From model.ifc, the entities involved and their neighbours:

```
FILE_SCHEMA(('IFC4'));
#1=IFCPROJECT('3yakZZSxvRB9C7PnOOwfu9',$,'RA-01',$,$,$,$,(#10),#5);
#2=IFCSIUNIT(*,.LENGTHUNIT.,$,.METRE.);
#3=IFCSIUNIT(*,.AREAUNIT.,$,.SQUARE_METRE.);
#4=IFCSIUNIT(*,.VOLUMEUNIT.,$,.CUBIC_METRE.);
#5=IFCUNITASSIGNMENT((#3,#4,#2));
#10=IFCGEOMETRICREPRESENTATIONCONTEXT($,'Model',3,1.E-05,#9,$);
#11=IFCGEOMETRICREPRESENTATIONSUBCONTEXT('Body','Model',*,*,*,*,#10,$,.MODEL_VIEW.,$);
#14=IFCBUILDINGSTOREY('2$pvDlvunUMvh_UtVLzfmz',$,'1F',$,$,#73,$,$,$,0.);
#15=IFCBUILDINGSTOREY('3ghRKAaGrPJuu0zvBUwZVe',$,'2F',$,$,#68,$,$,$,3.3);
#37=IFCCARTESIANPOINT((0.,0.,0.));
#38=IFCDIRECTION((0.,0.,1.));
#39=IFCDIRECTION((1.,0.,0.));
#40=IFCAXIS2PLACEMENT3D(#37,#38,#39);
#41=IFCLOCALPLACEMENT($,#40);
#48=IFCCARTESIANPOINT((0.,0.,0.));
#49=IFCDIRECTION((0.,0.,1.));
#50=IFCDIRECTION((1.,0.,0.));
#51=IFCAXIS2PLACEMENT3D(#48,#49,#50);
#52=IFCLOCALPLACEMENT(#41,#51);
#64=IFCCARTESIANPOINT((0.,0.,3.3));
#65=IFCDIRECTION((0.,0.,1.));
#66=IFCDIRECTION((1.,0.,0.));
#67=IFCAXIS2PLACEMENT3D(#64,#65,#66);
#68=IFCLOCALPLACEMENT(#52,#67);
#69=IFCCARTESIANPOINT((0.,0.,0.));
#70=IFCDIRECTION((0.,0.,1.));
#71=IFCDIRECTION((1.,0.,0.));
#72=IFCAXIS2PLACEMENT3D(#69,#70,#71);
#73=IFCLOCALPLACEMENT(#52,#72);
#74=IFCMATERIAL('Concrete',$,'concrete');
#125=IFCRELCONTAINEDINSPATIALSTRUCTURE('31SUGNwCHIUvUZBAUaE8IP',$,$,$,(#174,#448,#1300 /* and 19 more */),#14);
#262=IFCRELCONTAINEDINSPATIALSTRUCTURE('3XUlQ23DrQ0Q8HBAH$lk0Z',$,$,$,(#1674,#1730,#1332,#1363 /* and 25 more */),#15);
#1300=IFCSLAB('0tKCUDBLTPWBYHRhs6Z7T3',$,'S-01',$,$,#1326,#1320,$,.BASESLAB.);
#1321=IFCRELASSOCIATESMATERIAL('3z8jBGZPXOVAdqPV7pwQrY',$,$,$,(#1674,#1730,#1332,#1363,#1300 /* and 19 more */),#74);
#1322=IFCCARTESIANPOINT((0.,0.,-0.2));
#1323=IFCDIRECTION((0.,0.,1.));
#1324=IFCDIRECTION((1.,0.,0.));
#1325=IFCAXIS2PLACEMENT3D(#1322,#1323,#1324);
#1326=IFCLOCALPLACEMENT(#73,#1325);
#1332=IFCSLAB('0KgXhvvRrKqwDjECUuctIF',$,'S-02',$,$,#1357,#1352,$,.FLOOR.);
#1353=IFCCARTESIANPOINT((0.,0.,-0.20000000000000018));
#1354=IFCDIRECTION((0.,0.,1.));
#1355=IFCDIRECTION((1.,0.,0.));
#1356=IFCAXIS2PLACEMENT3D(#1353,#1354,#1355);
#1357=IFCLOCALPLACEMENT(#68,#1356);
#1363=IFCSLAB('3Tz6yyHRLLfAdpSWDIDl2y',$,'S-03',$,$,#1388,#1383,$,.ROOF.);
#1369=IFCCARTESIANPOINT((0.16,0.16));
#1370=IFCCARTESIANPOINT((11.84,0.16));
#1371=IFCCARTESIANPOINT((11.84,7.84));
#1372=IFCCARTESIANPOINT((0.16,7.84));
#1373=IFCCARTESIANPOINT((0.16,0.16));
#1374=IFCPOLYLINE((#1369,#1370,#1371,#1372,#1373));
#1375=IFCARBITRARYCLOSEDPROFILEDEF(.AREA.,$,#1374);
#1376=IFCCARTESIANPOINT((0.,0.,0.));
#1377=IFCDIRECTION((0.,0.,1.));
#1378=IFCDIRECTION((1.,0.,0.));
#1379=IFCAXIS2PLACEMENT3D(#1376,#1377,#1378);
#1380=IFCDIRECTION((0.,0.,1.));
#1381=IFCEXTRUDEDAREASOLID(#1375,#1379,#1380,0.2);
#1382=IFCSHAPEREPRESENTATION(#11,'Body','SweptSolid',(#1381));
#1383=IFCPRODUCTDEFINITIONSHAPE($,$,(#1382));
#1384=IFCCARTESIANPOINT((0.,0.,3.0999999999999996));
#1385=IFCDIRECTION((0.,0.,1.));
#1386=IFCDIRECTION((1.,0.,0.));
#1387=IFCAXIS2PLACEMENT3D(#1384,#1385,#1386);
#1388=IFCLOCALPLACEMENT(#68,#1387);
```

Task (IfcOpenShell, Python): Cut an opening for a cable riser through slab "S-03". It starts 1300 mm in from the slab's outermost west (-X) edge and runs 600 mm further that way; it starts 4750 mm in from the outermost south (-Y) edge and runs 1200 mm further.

```python
import numpy as np
import ifcopenshell
import ifcopenshell.api.feature
import ifcopenshell.api.geometry
import ifcopenshell.api.root
import ifcopenshell.geom
import ifcopenshell.util.placement
import ifcopenshell.util.representation
import ifcopenshell.util.shape
import ifcopenshell.util.unit

model = ifcopenshell.open("model.ifc")
unit_scale = ifcopenshell.util.unit.calculate_unit_scale(model)
settings = ifcopenshell.geom.settings()


def volume(element):
    """Net volume in cubic metres, openings subtracted."""
    shape = ifcopenshell.geom.create_shape(settings, element)
    return ifcopenshell.util.shape.get_volume(shape.geometry)


slab = model.by_guid("3Tz6yyHRLLfAdpSWDIDl2y")
before = volume(slab)

# Extent in the slab's own axes, in metres. The edges named are its -X and -Y sides.
slab_shape = ifcopenshell.geom.create_shape(settings, slab)
vertices = ifcopenshell.util.shape.get_vertices(slab_shape.geometry)
x_min, y_min, bottom = vertices.min(axis=0)
top = vertices[:, 2].max()

opening = ifcopenshell.api.root.create_entity(model, ifc_class="IfcOpeningElement", name="Cable riser opening", predefined_type="OPENING")
context = ifcopenshell.util.representation.get_context(model, "Model", "Body", "MODEL_VIEW")
width, depth = 0.6, 1.2
outline = [(0.0, 0.0), (width, 0.0), (width, depth), (0.0, depth), (0.0, 0.0)]
# Overshoot both faces by 50 mm so the cut is clean.
shape = ifcopenshell.api.geometry.add_slab_representation(
    model, context=context, depth=top - bottom + 0.1, polyline=outline
)
ifcopenshell.api.geometry.assign_representation(model, product=opening, representation=shape)

matrix = ifcopenshell.util.placement.get_local_placement(slab.ObjectPlacement)
matrix[:, 3] = matrix @ np.append(np.array([x_min + 1.3, y_min + 4.75, bottom - 0.05]) / unit_scale, 1.0)
ifcopenshell.api.geometry.edit_object_placement(model, product=opening, matrix=matrix, is_si=False)
ifcopenshell.api.feature.add_feature(model, feature=opening, element=slab)

after = volume(slab)

print(f"slab volume {before:.3f} -> {after:.3f} m3")

model.write("model_updated.ifc")
```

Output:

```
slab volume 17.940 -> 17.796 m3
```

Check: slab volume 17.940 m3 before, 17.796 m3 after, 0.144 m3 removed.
